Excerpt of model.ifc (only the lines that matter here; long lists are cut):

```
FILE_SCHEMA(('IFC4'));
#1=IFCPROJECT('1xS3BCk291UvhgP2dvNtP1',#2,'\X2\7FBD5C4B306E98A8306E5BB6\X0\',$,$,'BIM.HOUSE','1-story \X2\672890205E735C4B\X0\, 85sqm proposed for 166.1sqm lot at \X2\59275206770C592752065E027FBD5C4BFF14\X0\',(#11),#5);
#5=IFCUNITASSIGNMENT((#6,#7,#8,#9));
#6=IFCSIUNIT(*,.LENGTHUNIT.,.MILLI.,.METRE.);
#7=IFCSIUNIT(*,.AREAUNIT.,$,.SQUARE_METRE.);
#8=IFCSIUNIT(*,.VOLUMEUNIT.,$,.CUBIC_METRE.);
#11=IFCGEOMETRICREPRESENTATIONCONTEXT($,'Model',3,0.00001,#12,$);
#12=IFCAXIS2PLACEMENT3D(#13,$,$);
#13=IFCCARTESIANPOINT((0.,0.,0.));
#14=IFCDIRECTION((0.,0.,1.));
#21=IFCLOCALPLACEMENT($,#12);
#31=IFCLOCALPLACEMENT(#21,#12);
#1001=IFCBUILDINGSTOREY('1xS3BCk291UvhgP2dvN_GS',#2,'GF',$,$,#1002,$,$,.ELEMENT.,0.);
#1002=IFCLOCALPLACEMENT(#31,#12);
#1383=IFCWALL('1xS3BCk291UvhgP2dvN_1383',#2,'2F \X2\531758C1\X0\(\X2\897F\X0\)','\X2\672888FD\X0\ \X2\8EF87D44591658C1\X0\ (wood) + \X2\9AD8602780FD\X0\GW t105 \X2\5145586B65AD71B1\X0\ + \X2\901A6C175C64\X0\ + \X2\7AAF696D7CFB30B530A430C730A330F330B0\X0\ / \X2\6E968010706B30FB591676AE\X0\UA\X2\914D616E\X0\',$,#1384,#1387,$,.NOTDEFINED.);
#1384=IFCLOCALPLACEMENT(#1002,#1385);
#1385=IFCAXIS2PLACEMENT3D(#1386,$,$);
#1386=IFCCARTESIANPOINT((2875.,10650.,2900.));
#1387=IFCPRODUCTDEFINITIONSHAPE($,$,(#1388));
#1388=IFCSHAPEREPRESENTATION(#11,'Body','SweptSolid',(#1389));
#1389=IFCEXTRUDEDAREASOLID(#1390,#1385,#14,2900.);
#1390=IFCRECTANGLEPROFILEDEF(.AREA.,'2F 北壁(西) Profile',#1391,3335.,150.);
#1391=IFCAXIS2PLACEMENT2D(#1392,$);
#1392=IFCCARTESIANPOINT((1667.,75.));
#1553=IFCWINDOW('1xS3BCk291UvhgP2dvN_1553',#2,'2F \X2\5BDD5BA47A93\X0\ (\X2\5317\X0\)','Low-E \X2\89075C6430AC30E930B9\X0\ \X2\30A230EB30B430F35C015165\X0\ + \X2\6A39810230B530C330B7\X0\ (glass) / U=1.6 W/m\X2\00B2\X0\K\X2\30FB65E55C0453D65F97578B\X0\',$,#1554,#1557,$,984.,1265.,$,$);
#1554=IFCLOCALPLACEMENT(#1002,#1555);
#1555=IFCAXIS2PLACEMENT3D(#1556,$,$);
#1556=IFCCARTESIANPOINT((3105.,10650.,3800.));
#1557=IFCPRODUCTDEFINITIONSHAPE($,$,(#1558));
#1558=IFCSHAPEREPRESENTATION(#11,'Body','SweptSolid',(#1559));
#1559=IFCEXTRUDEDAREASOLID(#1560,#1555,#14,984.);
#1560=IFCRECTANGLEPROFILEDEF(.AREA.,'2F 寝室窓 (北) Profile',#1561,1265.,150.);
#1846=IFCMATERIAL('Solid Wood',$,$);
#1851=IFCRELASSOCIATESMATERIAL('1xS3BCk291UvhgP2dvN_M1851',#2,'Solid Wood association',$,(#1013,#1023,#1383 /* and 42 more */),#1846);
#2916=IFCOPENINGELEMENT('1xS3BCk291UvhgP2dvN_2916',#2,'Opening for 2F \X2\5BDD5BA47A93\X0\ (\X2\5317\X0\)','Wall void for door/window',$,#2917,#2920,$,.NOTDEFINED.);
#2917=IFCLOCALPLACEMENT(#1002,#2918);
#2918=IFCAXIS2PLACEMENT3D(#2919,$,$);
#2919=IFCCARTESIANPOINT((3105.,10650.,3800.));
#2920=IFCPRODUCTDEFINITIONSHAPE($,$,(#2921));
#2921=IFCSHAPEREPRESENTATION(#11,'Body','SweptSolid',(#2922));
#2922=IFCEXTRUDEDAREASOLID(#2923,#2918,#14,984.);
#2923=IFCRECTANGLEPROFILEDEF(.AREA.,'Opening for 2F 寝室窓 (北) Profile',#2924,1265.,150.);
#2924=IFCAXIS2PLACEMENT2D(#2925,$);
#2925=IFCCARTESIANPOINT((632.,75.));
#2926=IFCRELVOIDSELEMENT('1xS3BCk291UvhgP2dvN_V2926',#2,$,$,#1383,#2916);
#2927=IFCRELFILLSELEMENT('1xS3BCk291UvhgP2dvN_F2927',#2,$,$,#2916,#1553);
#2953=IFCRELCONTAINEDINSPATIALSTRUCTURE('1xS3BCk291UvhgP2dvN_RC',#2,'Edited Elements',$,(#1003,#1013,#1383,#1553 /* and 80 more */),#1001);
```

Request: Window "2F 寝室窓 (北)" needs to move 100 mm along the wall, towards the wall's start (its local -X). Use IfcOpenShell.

```python
import ifcopenshell
import ifcopenshell.api.geometry
import ifcopenshell.util.placement
import ifcopenshell.util.unit

model = ifcopenshell.open("model.ifc")
unit_scale = ifcopenshell.util.unit.calculate_unit_scale(model)

window = model.by_guid("1xS3BCk291UvhgP2dvN_1553")
opening = window.FillsVoids[0].RelatingOpeningElement
wall = opening.VoidsElements[0].RelatingBuildingElement

wall_matrix = ifcopenshell.util.placement.get_local_placement(wall.ObjectPlacement)
shift = wall_matrix[:3, 0] * -0.1 / unit_scale
before = ifcopenshell.util.placement.get_local_placement(window.ObjectPlacement)[:3, 3].copy()

# The window is not placed relative to its opening, so move both.
for product in (opening, window):
    matrix = ifcopenshell.util.placement.get_local_placement(product.ObjectPlacement)
    matrix[:3, 3] += shift
    ifcopenshell.api.geometry.edit_object_placement(model, product=product, matrix=matrix, is_si=False)

after = ifcopenshell.util.placement.get_local_placement(window.ObjectPlacement)[:3, 3]
print("window moved by", (after - before).round(3) + 0.0)

model.write("model_v2.ifc")
```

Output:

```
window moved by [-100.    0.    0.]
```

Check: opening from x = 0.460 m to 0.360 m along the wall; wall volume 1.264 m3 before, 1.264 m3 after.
